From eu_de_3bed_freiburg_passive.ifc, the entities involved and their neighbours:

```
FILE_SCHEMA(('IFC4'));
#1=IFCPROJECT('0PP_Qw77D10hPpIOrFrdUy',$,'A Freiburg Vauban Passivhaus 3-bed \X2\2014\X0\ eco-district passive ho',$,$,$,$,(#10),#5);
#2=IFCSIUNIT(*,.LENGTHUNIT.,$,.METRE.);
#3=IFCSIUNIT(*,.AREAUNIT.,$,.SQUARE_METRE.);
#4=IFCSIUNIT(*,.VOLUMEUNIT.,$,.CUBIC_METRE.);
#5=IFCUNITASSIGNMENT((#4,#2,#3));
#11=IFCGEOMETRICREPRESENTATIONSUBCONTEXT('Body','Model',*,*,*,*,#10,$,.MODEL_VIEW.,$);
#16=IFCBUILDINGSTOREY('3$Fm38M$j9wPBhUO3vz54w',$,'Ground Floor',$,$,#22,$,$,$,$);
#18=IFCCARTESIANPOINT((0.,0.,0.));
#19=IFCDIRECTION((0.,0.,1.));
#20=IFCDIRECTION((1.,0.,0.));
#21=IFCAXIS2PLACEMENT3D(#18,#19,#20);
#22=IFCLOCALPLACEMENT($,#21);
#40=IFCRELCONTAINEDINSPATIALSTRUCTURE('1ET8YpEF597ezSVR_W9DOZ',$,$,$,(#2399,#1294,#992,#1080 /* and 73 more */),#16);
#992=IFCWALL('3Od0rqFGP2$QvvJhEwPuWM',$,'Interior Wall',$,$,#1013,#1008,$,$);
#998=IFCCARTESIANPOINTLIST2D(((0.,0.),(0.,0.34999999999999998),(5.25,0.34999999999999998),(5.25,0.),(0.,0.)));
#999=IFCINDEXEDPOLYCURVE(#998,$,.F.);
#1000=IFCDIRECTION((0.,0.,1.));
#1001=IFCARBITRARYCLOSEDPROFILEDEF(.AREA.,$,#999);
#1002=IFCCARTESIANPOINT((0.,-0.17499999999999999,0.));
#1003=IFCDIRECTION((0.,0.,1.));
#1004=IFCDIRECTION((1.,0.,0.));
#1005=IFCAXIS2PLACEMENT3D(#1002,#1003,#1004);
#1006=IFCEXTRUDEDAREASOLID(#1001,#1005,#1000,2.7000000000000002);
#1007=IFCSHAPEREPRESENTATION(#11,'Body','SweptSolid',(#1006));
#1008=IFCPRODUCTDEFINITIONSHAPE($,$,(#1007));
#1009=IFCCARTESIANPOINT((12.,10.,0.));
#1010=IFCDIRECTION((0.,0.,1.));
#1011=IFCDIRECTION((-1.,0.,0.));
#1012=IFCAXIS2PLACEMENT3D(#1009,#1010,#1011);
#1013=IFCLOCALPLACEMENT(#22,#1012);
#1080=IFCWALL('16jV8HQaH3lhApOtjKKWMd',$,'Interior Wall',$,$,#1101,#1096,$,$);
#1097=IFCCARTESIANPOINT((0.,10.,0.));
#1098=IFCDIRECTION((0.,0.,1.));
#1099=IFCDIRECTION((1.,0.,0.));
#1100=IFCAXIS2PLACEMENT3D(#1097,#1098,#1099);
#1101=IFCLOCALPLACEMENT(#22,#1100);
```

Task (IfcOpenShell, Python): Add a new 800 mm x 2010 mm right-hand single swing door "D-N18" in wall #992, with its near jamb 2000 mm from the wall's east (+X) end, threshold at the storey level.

```python
import numpy as np
import ifcopenshell
import ifcopenshell.api.feature
import ifcopenshell.api.geometry
import ifcopenshell.api.root
import ifcopenshell.api.spatial
import ifcopenshell.geom
import ifcopenshell.util.element
import ifcopenshell.util.placement
import ifcopenshell.util.representation
import ifcopenshell.util.shape
import ifcopenshell.util.unit

model = ifcopenshell.open("eu_de_3bed_freiburg_passive.ifc")
unit_scale = ifcopenshell.util.unit.calculate_unit_scale(model)
settings = ifcopenshell.geom.settings()


def volume(element):
    """Net volume in cubic metres, openings subtracted."""
    shape = ifcopenshell.geom.create_shape(settings, element)
    return ifcopenshell.util.shape.get_volume(shape.geometry)


wall = model.by_guid("3Od0rqFGP2$QvvJhEwPuWM")
storey = ifcopenshell.util.element.get_container(wall, ifc_class="IfcBuildingStorey")
context = ifcopenshell.util.representation.get_context(model, "Model", "Body", "MODEL_VIEW")
before = volume(wall)

width, height, from_end, sill = 0.8, 2.01, 2, 0.0  # metres

# The wall runs along its own X axis, and the end named is its -X end.
wall_shape = ifcopenshell.geom.create_shape(settings, wall)
x, y, z = ifcopenshell.util.shape.get_vertices(wall_shape.geometry).T
start = x.min() + from_end
face, thickness = float(y.min()), float(y.max() - y.min())
wall_matrix = ifcopenshell.util.placement.get_local_placement(wall.ObjectPlacement)
level = ifcopenshell.util.placement.get_local_placement(storey.ObjectPlacement)[2, 3]


def in_wall(x, y):
    """Placement at x, y metres in the wall's axes, at sill height."""
    matrix = wall_matrix.copy()
    matrix[:, 3] = wall_matrix @ np.array([x / unit_scale, y / unit_scale, 0.0, 1.0])
    matrix[2, 3] = level + sill / unit_scale
    return matrix


# Opening: a box that overshoots both wall faces by 50 mm.
opening = ifcopenshell.api.root.create_entity(model, ifc_class="IfcOpeningElement", predefined_type="OPENING")
box = ifcopenshell.api.geometry.add_wall_representation(
    model, context=context, length=width, height=height, thickness=thickness + 0.1
)
ifcopenshell.api.geometry.assign_representation(model, product=opening, representation=box)
ifcopenshell.api.geometry.edit_object_placement(model, product=opening, matrix=in_wall(start, face - 0.05), is_si=False)
ifcopenshell.api.feature.add_feature(model, feature=opening, element=wall)

door = ifcopenshell.api.root.create_entity(model, ifc_class="IfcDoor", name="D-N18", predefined_type="DOOR")
door.OverallWidth, door.OverallHeight = width / unit_scale, height / unit_scale
door.OperationType = "SINGLE_SWING_RIGHT"
body = ifcopenshell.api.geometry.add_door_representation(
    model,
    context=context,
    overall_width=door.OverallWidth,
    overall_height=door.OverallHeight,
    operation_type="SINGLE_SWING_RIGHT",
    lining_properties={"LiningDepth": thickness / unit_scale, "ThresholdDepth": thickness / unit_scale},
)
ifcopenshell.api.geometry.assign_representation(model, product=door, representation=body)
ifcopenshell.api.spatial.assign_container(model, products=[door], relating_structure=storey)
ifcopenshell.api.feature.add_filling(model, opening=opening, element=door)

# The lining spans the wall, so the door starts at the wall face.
ifcopenshell.api.geometry.edit_object_placement(model, product=door, matrix=in_wall(start, face), is_si=False)

after = volume(wall)

print(f"wall volume {before:.3f} -> {after:.3f} m3")

model.write("eu_de_3bed_freiburg_passive_v2.ifc")
```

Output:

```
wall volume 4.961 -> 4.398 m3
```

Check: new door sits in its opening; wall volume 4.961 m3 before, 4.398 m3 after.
